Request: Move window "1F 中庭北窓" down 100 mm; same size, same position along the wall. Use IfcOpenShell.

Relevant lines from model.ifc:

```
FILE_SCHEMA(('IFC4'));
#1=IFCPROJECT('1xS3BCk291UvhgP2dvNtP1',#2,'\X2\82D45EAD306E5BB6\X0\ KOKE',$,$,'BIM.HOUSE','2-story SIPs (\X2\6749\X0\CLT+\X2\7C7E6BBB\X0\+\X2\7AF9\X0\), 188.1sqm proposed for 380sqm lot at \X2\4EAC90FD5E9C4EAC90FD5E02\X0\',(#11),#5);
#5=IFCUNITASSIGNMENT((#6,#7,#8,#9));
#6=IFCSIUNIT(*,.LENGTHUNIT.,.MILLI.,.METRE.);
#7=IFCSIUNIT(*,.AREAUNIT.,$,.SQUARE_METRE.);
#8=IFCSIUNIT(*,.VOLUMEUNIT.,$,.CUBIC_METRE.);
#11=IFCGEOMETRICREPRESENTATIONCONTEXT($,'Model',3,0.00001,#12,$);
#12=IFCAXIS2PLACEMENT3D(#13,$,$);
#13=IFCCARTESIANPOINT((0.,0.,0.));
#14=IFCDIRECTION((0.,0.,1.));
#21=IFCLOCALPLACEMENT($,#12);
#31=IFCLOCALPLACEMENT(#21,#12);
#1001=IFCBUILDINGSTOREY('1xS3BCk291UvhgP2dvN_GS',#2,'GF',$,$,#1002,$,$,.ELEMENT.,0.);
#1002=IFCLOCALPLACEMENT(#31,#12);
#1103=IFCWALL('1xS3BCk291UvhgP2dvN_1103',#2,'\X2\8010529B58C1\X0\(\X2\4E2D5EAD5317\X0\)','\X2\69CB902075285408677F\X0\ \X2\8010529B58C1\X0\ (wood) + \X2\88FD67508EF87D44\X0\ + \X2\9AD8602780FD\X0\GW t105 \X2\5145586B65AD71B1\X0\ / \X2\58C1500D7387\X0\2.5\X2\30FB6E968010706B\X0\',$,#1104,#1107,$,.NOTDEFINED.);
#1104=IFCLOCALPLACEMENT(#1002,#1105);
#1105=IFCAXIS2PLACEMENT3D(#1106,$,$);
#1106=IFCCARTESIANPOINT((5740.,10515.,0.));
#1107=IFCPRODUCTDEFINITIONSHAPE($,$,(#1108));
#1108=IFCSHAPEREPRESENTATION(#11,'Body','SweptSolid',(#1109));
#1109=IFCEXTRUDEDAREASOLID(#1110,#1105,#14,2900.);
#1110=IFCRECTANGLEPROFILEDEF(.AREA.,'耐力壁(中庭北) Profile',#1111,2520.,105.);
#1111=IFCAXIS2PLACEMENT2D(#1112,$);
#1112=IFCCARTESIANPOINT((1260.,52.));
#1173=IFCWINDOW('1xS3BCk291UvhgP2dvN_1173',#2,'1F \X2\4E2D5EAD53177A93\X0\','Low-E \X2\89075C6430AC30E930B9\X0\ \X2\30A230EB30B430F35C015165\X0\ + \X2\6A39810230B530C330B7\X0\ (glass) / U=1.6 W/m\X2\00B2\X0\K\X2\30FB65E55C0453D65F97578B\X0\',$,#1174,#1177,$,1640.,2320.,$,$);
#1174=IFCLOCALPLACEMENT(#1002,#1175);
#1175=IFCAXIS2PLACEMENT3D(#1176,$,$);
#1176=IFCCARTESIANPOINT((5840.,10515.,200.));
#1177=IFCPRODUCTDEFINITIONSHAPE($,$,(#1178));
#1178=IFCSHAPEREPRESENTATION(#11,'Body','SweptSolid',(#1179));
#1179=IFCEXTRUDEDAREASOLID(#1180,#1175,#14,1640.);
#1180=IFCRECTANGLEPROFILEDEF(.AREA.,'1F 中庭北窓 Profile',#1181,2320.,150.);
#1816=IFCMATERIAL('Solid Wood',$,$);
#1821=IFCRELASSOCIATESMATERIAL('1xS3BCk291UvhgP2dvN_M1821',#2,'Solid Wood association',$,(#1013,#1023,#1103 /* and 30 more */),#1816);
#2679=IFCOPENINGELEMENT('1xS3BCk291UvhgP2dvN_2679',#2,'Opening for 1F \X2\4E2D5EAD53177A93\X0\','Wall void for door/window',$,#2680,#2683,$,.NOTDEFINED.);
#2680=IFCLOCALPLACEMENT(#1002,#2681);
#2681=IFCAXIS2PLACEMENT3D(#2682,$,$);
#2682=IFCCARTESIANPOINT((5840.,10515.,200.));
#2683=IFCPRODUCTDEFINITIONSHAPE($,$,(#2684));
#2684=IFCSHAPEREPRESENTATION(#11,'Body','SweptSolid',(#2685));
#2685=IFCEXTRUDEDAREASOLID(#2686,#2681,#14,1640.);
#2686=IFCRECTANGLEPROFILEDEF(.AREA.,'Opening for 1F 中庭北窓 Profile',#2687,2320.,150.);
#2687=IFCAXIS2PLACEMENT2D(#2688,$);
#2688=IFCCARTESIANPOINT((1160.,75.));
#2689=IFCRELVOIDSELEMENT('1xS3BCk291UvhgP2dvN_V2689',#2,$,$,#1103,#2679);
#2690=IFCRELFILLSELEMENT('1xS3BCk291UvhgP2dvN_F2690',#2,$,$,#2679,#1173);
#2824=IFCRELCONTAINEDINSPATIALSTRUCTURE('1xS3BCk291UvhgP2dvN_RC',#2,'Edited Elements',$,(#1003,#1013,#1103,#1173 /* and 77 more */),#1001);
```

```python
import numpy as np
import ifcopenshell
import ifcopenshell.api.geometry
import ifcopenshell.util.placement
import ifcopenshell.util.unit

model = ifcopenshell.open("model.ifc")
unit_scale = ifcopenshell.util.unit.calculate_unit_scale(model)

window = model.by_guid("1xS3BCk291UvhgP2dvN_1173")
opening = window.FillsVoids[0].RelatingOpeningElement
dz = -100.0

shift = np.array([0.0, 0.0, dz])
# The window is not placed relative to its opening, so move both.
for product in (opening, window):
    matrix = ifcopenshell.util.placement.get_local_placement(product.ObjectPlacement)
    matrix[:3, 3] += shift
    ifcopenshell.api.geometry.edit_object_placement(model, product=product, matrix=matrix, is_si=False)

print(f"moved by {dz * unit_scale:+.3f} m")

model.write("model_edited.ifc")
```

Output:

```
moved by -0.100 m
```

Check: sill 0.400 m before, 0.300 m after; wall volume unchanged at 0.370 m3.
